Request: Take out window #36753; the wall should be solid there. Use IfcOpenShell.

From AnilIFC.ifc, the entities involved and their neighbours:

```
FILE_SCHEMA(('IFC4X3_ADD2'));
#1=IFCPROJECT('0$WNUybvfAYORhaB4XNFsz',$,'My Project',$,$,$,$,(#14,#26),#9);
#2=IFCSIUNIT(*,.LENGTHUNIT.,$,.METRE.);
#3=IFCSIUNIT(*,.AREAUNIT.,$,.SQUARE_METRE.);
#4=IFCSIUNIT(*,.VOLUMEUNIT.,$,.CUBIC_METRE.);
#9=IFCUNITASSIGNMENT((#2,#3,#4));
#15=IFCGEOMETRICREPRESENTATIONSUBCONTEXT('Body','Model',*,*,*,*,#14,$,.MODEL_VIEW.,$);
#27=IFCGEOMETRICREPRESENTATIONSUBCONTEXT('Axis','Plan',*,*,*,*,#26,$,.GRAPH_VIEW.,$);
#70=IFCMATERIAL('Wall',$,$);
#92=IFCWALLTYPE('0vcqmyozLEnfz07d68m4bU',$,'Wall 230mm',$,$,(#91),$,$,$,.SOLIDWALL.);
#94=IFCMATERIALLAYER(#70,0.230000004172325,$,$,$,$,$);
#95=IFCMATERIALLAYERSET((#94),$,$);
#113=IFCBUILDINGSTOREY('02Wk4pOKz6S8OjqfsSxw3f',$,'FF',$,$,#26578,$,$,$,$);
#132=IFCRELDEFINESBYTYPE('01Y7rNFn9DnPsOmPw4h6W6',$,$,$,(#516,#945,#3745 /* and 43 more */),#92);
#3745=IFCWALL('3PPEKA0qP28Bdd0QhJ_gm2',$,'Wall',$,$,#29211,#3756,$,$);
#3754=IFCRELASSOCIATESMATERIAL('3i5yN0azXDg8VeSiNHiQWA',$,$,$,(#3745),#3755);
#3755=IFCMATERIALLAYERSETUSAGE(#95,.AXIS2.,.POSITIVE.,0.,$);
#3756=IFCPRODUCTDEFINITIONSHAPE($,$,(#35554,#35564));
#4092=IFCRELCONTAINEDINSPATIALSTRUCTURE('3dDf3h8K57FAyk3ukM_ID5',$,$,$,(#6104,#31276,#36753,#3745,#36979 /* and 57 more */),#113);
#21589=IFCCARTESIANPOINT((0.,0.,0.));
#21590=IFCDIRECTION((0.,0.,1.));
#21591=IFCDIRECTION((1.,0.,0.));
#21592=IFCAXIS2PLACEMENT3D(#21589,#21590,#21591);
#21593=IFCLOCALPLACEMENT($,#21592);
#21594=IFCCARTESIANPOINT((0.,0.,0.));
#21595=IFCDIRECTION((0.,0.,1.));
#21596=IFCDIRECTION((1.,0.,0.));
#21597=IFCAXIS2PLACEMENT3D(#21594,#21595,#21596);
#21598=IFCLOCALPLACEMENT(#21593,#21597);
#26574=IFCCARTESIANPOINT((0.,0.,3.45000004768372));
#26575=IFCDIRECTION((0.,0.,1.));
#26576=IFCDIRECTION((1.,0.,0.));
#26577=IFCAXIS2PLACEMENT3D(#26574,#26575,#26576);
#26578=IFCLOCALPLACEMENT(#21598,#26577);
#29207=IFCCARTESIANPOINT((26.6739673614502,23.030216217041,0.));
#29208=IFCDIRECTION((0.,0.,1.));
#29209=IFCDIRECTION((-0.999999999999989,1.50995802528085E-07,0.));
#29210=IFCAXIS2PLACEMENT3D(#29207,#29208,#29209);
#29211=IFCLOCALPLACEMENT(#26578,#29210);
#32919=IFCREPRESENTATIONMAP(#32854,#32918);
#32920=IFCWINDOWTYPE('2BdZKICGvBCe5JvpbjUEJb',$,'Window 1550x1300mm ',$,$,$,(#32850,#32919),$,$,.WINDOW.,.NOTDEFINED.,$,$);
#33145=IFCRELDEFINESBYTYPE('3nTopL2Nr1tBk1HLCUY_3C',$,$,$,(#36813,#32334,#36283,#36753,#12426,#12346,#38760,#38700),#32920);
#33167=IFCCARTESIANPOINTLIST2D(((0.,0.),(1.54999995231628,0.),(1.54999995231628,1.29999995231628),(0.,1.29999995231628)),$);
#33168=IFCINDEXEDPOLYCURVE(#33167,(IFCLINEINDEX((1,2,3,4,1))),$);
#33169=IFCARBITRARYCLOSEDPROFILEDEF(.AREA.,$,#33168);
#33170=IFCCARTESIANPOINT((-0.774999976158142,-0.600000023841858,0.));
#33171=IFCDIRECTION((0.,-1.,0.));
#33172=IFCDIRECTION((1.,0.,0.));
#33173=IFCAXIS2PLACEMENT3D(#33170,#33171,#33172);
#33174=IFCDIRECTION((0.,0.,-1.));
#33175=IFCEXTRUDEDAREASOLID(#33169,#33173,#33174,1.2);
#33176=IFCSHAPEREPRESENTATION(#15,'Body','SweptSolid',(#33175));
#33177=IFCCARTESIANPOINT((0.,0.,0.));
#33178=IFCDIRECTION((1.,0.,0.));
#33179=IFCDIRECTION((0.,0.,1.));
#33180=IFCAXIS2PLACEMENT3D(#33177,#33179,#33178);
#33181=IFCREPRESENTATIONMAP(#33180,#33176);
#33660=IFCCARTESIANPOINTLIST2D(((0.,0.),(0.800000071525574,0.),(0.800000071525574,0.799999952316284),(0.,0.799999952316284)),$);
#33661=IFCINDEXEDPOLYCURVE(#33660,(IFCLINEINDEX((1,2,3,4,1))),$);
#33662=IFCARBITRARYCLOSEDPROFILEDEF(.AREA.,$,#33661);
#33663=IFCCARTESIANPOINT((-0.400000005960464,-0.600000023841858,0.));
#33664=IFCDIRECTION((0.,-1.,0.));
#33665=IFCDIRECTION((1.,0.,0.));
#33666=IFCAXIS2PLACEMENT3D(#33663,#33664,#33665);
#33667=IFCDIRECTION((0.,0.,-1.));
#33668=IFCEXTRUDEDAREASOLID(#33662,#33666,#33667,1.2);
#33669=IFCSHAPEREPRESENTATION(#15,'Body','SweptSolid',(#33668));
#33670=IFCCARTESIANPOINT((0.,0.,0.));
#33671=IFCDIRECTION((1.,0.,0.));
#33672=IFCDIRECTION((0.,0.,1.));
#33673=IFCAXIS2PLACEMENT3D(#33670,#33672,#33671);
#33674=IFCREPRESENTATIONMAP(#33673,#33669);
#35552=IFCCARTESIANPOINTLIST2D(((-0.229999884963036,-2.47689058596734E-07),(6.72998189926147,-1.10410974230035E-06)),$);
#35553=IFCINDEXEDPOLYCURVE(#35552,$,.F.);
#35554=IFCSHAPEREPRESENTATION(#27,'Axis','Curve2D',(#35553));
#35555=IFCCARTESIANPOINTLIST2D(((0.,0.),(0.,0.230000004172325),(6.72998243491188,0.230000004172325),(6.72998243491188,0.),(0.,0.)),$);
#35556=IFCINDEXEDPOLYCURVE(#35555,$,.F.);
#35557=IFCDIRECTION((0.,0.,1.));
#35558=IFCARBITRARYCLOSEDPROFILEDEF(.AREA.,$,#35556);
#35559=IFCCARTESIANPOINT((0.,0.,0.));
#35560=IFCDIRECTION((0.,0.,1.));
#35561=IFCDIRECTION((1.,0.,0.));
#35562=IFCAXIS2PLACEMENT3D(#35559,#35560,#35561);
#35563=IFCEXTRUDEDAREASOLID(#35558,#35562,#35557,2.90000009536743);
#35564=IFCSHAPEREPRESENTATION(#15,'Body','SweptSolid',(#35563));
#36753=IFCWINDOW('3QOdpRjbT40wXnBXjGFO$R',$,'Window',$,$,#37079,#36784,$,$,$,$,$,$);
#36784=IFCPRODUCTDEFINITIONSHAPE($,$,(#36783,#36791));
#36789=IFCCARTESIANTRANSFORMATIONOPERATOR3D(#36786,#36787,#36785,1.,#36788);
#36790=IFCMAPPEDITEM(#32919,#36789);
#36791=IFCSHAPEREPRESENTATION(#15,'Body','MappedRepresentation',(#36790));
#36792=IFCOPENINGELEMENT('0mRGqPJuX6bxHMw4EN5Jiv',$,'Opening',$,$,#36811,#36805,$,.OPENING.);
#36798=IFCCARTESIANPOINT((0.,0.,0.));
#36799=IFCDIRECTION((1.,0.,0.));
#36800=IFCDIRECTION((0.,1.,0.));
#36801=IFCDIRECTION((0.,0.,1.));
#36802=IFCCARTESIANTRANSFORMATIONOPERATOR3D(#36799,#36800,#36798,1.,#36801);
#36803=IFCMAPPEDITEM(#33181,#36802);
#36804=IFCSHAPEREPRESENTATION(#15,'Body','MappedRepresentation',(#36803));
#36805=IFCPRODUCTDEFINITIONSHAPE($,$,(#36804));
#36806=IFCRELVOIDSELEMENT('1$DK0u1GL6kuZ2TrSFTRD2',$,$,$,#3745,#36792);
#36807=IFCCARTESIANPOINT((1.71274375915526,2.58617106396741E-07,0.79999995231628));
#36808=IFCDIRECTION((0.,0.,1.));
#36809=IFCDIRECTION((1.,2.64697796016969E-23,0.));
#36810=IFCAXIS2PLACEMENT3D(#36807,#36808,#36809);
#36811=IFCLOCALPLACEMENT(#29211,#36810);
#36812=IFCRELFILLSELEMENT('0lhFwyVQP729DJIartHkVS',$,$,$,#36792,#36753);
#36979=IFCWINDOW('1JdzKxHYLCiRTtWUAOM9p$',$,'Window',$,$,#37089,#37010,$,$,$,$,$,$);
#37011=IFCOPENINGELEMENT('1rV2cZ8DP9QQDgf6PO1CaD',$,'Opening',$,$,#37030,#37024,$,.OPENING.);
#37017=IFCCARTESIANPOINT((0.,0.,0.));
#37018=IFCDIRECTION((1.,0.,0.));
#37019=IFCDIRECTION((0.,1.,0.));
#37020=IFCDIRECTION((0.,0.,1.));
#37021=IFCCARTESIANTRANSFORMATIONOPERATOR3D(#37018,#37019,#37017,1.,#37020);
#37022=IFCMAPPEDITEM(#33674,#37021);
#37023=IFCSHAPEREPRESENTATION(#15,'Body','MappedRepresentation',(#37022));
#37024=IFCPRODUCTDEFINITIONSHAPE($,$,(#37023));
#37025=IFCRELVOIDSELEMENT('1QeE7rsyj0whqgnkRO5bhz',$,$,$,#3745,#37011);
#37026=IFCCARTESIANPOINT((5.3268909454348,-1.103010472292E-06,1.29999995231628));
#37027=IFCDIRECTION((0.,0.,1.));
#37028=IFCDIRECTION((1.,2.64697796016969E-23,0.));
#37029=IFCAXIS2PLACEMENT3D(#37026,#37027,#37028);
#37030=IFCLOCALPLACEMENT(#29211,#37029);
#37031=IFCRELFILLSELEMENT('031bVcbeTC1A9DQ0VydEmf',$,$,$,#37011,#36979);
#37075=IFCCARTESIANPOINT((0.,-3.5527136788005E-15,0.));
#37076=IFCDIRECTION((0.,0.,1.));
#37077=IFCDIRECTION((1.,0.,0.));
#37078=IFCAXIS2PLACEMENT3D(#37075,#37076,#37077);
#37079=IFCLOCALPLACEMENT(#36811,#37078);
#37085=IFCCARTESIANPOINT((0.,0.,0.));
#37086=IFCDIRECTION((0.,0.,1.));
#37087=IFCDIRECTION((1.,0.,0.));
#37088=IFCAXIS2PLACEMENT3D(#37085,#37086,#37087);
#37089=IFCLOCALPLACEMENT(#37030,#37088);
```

```python
import ifcopenshell
import ifcopenshell.api.feature
import ifcopenshell.api.root
import ifcopenshell.geom
import ifcopenshell.util.shape

model = ifcopenshell.open("AnilIFC.ifc")
settings = ifcopenshell.geom.settings()


def volume(element):
    """Net volume in cubic metres, openings subtracted."""
    shape = ifcopenshell.geom.create_shape(settings, element)
    return ifcopenshell.util.shape.get_volume(shape.geometry)


window = model.by_id(36753)
opening = window.FillsVoids[0].RelatingOpeningElement
wall = opening.VoidsElements[0].RelatingBuildingElement
before = volume(wall)

ifcopenshell.api.root.remove_product(model, product=window)
ifcopenshell.api.feature.remove_feature(model, feature=opening)

after = volume(wall)

print(f"wall volume {before:.3f} -> {after:.3f} m3")

model.write("AnilIFC_rev.ifc")
```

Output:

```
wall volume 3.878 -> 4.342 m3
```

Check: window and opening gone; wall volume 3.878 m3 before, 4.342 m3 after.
